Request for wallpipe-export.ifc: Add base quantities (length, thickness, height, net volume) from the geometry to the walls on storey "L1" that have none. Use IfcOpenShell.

First a look at what the model holds.

```python
import ifcopenshell
import ifcopenshell.util.element
import ifcopenshell.util.unit

model = ifcopenshell.open("wallpipe-export.ifc")
print(model.schema)
for unit_type in ("LENGTHUNIT", "AREAUNIT", "VOLUMEUNIT"):
    print(unit_type, ifcopenshell.util.unit.calculate_unit_scale(model, unit_type))
storey = next(s for s in model.by_type("IfcBuildingStorey") if s.Name == "L1")
walls = [e for e in ifcopenshell.util.element.get_decomposition(storey) if e.is_a("IfcWall")]
for e in sorted(walls, key=lambda e: e.id()):
    print(e.id(), e.is_a(), e.Name, list(ifcopenshell.util.element.get_psets(e, qtos_only=True)), sep=" | ")
```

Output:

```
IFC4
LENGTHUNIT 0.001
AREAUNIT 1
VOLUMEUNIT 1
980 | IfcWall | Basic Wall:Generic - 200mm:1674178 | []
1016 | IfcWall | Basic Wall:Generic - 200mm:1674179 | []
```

```python
import ifcopenshell
import ifcopenshell.api.pset
import ifcopenshell.geom
import ifcopenshell.util.element
import ifcopenshell.util.shape
import ifcopenshell.util.unit

model = ifcopenshell.open("wallpipe-export.ifc")
unit_scale = ifcopenshell.util.unit.calculate_unit_scale(model)
volume_scale = ifcopenshell.util.unit.calculate_unit_scale(model, "VOLUMEUNIT")
settings = ifcopenshell.geom.settings()

storey = next(s for s in model.by_type("IfcBuildingStorey") if s.Name == "L1")
walls = [e for e in ifcopenshell.util.element.get_decomposition(storey) if e.is_a("IfcWall")]

for e in sorted(walls, key=lambda e: e.id()):
    if ifcopenshell.util.element.get_psets(e, qtos_only=True, should_inherit=False):
        continue
    # Geometry comes back in metres, in the element's own axes.
    shape = ifcopenshell.geom.create_shape(settings, e)
    values = {
        "Length": ifcopenshell.util.shape.get_x(shape.geometry) / unit_scale,
        "Width": ifcopenshell.util.shape.get_y(shape.geometry) / unit_scale,
        "Height": ifcopenshell.util.shape.get_z(shape.geometry) / unit_scale,
        "NetVolume": ifcopenshell.util.shape.get_volume(shape.geometry) / volume_scale,
    }
    qto = ifcopenshell.api.pset.add_qto(model, product=e, name="Qto_WallBaseQuantities")
    ifcopenshell.api.pset.edit_qto(model, qto=qto, properties=values)
    print(e.id(), {k: round(v, 3) for k, v in values.items()})

model.write("wallpipe-export_rev.ifc")
```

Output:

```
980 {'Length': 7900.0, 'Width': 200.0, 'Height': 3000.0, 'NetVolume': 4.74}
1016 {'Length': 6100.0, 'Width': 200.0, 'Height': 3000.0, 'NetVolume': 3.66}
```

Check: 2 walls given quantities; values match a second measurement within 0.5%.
